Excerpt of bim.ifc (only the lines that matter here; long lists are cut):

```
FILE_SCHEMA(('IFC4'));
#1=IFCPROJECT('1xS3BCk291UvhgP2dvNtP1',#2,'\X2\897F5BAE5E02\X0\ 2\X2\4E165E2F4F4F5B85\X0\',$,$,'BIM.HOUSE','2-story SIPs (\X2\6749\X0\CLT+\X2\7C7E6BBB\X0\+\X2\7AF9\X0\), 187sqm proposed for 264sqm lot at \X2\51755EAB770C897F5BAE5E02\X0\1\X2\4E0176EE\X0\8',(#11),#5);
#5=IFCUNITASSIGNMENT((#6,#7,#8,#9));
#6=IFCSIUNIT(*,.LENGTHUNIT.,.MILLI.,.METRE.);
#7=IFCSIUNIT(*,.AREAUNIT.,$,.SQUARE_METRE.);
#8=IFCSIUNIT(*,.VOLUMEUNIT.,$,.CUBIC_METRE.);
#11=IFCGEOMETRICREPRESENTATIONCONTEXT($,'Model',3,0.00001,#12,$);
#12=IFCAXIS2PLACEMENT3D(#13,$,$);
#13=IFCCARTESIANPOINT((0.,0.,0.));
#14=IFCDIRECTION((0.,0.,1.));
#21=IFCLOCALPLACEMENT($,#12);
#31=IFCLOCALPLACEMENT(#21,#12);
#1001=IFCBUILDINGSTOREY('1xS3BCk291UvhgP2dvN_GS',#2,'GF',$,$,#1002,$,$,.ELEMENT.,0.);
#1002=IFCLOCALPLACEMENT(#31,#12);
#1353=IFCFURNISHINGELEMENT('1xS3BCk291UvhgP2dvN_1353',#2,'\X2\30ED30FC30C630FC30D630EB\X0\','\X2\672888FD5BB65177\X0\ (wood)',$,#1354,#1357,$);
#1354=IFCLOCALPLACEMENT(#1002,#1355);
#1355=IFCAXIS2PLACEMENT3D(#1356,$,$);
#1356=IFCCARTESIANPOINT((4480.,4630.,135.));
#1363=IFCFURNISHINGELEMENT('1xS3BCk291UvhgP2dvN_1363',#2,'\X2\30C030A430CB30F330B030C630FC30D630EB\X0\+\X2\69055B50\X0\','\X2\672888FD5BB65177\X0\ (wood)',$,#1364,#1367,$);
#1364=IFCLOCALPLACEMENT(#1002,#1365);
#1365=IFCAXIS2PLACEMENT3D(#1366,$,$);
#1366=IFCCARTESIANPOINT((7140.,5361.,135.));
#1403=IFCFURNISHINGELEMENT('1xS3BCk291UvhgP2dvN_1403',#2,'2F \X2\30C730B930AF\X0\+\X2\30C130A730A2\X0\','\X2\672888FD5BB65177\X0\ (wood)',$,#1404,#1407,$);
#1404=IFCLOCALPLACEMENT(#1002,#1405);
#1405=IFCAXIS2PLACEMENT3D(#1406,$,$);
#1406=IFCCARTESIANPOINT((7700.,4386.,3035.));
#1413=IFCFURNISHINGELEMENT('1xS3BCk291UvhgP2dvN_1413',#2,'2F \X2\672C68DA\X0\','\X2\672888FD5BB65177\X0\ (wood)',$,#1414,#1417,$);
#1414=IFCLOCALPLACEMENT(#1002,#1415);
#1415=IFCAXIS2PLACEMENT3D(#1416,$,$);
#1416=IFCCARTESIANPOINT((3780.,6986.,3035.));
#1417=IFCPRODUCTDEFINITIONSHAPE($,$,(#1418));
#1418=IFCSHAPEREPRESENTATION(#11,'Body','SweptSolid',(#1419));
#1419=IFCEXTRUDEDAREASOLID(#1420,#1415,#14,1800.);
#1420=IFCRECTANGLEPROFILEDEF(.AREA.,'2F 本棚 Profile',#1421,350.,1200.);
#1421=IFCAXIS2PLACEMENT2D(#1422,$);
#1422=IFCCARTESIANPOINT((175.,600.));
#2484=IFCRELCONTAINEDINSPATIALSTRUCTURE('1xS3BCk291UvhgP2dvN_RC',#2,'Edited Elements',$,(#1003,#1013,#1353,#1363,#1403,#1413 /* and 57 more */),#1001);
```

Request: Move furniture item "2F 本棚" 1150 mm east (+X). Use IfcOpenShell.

```python
import ifcopenshell
import ifcopenshell.api.geometry
import ifcopenshell.util.placement

model = ifcopenshell.open("bim.ifc")

item = model.by_id(1413)
matrix = ifcopenshell.util.placement.get_local_placement(item.ObjectPlacement)
matrix[0, 3] += 1150.0
ifcopenshell.api.geometry.edit_object_placement(model, product=item, matrix=matrix, is_si=False)

print(ifcopenshell.util.placement.get_local_placement(item.ObjectPlacement).round(3) + 0.0)

model.write("bim_updated.ifc")
```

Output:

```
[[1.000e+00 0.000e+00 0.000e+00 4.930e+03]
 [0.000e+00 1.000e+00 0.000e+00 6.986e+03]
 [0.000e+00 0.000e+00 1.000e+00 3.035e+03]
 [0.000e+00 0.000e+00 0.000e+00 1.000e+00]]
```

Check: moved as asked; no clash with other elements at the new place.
